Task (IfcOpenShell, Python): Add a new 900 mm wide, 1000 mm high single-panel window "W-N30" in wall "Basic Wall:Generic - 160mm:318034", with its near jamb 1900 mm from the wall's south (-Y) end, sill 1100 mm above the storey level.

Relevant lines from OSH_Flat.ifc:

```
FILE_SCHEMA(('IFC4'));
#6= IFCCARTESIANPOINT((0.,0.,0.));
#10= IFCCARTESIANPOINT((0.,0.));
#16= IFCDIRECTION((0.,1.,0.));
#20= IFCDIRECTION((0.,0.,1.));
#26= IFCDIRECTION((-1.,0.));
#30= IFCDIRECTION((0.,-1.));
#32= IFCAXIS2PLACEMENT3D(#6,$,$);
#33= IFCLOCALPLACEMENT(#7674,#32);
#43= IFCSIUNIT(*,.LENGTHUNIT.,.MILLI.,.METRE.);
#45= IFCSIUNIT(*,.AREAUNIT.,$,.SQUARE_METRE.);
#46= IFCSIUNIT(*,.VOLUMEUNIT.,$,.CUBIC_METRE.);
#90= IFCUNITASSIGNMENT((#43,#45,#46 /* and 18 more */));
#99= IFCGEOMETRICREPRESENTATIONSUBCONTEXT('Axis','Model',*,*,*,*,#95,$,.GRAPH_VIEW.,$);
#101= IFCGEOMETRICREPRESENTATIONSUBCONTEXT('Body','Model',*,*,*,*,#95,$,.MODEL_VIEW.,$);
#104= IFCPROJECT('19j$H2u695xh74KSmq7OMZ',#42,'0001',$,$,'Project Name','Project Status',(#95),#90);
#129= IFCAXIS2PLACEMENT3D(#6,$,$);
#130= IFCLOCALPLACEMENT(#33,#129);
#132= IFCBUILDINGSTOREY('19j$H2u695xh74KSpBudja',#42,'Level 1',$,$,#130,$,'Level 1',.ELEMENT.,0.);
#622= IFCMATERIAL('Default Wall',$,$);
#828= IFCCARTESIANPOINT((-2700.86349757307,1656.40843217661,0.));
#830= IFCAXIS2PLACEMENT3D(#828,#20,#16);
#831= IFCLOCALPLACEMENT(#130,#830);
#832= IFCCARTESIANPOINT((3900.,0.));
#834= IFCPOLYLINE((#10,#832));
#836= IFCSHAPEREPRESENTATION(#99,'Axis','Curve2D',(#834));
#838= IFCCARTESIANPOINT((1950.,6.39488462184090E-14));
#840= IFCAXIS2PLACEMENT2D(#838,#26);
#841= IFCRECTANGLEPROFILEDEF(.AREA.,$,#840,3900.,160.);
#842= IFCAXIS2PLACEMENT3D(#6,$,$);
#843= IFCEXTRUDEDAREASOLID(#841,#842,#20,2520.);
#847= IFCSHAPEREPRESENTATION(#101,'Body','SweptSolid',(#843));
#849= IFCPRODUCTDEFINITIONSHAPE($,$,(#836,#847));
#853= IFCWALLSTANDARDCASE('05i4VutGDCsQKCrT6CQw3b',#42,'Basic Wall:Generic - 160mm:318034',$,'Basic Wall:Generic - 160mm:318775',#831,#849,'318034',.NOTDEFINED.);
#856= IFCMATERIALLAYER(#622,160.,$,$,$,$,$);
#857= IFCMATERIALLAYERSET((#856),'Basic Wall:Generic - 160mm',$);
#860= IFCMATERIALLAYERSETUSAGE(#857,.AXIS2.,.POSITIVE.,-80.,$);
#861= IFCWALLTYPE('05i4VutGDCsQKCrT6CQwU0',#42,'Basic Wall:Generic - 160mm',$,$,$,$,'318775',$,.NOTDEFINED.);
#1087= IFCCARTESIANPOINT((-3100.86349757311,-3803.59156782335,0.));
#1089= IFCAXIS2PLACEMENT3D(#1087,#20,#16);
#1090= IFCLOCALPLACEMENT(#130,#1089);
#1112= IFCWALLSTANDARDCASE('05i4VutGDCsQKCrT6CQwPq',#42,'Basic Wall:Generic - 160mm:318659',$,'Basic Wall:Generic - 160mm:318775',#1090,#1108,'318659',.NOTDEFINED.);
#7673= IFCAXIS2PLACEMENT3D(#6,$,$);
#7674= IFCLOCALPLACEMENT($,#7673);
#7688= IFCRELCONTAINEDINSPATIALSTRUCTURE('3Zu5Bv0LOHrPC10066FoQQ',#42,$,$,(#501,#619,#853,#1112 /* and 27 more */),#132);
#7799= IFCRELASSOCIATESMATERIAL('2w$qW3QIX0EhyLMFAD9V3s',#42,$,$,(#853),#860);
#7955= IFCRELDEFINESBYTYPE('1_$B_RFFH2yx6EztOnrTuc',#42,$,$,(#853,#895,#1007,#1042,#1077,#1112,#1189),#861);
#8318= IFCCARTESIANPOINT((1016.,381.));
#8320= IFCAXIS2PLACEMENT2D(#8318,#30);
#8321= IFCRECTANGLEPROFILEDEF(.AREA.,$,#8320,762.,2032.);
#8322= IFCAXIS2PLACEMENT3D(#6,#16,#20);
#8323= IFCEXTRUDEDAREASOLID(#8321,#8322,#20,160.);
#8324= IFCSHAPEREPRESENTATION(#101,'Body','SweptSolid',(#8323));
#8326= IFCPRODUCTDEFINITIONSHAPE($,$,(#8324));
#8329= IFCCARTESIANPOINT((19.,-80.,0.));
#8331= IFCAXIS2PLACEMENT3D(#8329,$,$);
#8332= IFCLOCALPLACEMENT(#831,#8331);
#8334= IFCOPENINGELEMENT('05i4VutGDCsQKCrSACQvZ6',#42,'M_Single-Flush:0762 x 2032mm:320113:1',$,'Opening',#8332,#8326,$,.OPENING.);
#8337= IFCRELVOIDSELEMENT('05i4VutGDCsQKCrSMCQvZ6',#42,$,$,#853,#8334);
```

```python
import numpy as np
import ifcopenshell
import ifcopenshell.api.feature
import ifcopenshell.api.geometry
import ifcopenshell.api.root
import ifcopenshell.api.spatial
import ifcopenshell.geom
import ifcopenshell.util.element
import ifcopenshell.util.placement
import ifcopenshell.util.representation
import ifcopenshell.util.shape
import ifcopenshell.util.unit

model = ifcopenshell.open("OSH_Flat.ifc")
unit_scale = ifcopenshell.util.unit.calculate_unit_scale(model)
settings = ifcopenshell.geom.settings()


def volume(element):
    """Net volume in cubic metres, openings subtracted."""
    shape = ifcopenshell.geom.create_shape(settings, element)
    return ifcopenshell.util.shape.get_volume(shape.geometry)


wall = model.by_id(853)
storey = ifcopenshell.util.element.get_container(wall, ifc_class="IfcBuildingStorey")
context = ifcopenshell.util.representation.get_context(model, "Model", "Body", "MODEL_VIEW")
before = volume(wall)

width, height, from_end, sill = 0.9, 1, 1.9, 1.1  # metres

# The wall runs along its own X axis, and the end named is its -X end.
wall_shape = ifcopenshell.geom.create_shape(settings, wall)
x, y, z = ifcopenshell.util.shape.get_vertices(wall_shape.geometry).T
start = x.min() + from_end
face, thickness = float(y.min()), float(y.max() - y.min())
wall_matrix = ifcopenshell.util.placement.get_local_placement(wall.ObjectPlacement)
level = ifcopenshell.util.placement.get_local_placement(storey.ObjectPlacement)[2, 3]


def in_wall(x, y):
    """Placement at x, y metres in the wall's axes, at sill height."""
    matrix = wall_matrix.copy()
    matrix[:, 3] = wall_matrix @ np.array([x / unit_scale, y / unit_scale, 0.0, 1.0])
    matrix[2, 3] = level + sill / unit_scale
    return matrix


# Opening: a box that overshoots both wall faces by 50 mm.
opening = ifcopenshell.api.root.create_entity(model, ifc_class="IfcOpeningElement", predefined_type="OPENING")
box = ifcopenshell.api.geometry.add_wall_representation(
    model, context=context, length=width, height=height, thickness=thickness + 0.1
)
ifcopenshell.api.geometry.assign_representation(model, product=opening, representation=box)
ifcopenshell.api.geometry.edit_object_placement(model, product=opening, matrix=in_wall(start, face - 0.05), is_si=False)
ifcopenshell.api.feature.add_feature(model, feature=opening, element=wall)

window = ifcopenshell.api.root.create_entity(model, ifc_class="IfcWindow", name="W-N30", predefined_type="WINDOW")
window.OverallWidth, window.OverallHeight = width / unit_scale, height / unit_scale
window.PartitioningType = "SINGLE_PANEL"
body = ifcopenshell.api.geometry.add_window_representation(
    model,
    context=context,
    overall_width=window.OverallWidth,
    overall_height=window.OverallHeight,
    partition_type="SINGLE_PANEL",
)
ifcopenshell.api.geometry.assign_representation(model, product=window, representation=body)
ifcopenshell.api.spatial.assign_container(model, products=[window], relating_structure=storey)
ifcopenshell.api.feature.add_filling(model, opening=opening, element=window)

# Centre the window in the wall's thickness.
ifcopenshell.api.geometry.edit_object_placement(model, product=window, matrix=in_wall(start, face), is_si=False)
window_shape = ifcopenshell.geom.create_shape(settings, window)
depth = ifcopenshell.util.shape.get_vertices(window_shape.geometry)[:, 1]
offset = face + thickness / 2 - (depth.min() + depth.max()) / 2
ifcopenshell.api.geometry.edit_object_placement(model, product=window, matrix=in_wall(start, offset), is_si=False)

after = volume(wall)

print(f"wall volume {before:.3f} -> {after:.3f} m3")

model.write("OSH_Flat_edited.ifc")
```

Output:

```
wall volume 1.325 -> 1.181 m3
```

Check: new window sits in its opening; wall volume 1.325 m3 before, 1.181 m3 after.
